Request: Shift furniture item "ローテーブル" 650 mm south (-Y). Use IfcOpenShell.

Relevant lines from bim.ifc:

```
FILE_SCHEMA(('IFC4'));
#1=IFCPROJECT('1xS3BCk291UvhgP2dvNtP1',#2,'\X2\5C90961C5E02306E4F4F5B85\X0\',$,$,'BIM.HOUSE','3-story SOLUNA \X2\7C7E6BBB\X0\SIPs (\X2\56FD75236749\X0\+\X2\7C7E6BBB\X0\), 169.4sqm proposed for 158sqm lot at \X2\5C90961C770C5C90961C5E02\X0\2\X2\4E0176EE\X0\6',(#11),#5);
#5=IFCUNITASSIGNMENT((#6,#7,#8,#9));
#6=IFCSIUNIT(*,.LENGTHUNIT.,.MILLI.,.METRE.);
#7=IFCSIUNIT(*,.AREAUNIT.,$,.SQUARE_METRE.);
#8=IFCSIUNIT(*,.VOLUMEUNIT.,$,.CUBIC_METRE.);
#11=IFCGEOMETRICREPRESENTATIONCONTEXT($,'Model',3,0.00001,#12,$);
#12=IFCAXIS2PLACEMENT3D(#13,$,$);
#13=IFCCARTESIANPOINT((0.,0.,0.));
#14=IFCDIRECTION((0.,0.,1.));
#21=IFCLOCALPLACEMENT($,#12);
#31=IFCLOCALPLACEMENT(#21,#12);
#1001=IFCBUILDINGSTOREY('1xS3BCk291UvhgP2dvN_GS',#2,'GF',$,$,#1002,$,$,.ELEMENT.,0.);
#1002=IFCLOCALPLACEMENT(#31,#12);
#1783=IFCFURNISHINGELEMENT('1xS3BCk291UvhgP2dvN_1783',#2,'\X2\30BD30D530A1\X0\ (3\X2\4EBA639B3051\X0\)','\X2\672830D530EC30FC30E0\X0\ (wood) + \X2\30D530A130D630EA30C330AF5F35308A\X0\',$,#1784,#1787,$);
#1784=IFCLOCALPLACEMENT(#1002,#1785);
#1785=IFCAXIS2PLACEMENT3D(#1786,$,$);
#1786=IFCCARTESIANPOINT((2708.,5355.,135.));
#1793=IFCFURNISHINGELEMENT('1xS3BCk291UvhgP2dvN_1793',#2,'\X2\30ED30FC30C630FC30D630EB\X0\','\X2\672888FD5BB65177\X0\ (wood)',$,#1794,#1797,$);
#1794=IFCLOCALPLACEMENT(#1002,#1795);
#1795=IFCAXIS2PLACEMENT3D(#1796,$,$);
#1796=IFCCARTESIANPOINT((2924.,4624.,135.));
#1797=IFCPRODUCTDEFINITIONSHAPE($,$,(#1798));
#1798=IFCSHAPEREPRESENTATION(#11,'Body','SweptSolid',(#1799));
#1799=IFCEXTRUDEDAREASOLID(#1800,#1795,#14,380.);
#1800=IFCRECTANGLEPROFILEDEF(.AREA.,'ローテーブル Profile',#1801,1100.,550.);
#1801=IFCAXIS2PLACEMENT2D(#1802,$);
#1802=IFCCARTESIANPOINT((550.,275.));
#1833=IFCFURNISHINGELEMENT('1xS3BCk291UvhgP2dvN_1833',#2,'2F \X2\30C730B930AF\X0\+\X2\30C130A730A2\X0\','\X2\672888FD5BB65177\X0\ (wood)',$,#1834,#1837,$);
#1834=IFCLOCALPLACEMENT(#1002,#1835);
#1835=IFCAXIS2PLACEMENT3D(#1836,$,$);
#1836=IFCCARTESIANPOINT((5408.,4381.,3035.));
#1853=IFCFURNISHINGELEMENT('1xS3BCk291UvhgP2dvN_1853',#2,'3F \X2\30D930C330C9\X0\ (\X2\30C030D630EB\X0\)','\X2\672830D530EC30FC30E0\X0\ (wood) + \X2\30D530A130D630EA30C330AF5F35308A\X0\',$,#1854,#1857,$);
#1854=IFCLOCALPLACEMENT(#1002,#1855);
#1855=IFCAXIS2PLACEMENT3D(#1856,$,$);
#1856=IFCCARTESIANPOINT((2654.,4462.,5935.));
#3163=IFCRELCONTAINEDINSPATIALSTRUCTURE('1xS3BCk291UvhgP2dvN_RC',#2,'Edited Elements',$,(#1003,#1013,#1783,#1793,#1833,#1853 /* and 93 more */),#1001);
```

```python
import ifcopenshell
import ifcopenshell.api.geometry
import ifcopenshell.util.placement

model = ifcopenshell.open("bim.ifc")

item = model.by_guid("1xS3BCk291UvhgP2dvN_1793")
matrix = ifcopenshell.util.placement.get_local_placement(item.ObjectPlacement)
matrix[1, 3] -= 650.0
ifcopenshell.api.geometry.edit_object_placement(model, product=item, matrix=matrix, is_si=False)

print(ifcopenshell.util.placement.get_local_placement(item.ObjectPlacement).round(3) + 0.0)

model.write("bim_rev.ifc")
```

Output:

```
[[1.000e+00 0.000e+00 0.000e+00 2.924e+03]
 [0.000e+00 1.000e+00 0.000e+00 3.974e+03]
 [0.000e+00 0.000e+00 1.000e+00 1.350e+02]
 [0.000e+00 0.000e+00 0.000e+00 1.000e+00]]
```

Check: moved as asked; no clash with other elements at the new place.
